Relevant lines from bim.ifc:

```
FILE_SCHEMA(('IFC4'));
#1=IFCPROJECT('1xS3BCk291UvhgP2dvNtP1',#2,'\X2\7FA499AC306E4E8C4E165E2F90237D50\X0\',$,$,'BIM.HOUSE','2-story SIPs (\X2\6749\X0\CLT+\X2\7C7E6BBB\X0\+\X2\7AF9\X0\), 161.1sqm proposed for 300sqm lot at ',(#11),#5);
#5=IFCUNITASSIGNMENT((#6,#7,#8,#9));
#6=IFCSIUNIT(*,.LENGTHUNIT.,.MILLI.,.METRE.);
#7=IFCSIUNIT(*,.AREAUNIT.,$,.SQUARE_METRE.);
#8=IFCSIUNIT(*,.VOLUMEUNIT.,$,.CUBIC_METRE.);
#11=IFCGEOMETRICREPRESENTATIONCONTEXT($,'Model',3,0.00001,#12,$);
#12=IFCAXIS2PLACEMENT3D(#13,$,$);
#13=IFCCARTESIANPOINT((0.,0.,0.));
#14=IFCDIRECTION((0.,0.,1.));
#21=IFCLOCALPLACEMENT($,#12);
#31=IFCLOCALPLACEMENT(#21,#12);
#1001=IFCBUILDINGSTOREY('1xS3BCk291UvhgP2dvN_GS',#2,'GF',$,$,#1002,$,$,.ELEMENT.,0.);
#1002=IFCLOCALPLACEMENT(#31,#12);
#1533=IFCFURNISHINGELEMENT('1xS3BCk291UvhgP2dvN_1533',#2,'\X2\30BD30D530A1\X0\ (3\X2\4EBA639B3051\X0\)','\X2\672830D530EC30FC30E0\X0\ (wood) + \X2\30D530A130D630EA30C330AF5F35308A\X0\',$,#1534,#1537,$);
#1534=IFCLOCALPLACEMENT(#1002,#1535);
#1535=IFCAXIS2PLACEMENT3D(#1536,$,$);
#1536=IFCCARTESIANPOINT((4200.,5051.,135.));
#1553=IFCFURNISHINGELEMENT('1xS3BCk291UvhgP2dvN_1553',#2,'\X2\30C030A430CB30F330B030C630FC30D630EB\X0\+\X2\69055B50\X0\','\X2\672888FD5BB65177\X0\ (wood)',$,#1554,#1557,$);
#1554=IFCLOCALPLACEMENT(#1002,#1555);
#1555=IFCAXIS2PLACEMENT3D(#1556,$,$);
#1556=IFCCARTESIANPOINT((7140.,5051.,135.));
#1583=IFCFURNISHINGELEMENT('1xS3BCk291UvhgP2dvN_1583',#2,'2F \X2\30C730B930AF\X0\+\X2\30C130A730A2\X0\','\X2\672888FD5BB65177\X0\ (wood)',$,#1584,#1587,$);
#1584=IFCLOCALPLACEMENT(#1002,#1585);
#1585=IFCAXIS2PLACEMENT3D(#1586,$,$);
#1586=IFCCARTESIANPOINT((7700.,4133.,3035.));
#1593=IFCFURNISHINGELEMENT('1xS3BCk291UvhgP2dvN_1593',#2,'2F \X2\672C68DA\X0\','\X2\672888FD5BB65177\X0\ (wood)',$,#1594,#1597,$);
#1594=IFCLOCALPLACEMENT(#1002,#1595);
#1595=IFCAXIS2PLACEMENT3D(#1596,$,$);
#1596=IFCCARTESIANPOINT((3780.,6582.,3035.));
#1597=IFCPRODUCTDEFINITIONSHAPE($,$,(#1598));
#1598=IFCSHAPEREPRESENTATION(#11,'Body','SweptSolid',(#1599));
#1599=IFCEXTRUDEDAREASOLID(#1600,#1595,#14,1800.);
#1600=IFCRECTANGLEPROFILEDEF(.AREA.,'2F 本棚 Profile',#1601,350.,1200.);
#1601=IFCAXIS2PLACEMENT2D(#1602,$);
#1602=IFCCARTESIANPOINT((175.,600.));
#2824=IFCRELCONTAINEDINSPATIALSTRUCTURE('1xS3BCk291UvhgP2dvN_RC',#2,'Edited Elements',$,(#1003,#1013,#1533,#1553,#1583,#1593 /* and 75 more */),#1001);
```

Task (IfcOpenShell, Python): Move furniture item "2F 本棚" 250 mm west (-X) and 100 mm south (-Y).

```python
import ifcopenshell
import ifcopenshell.api.geometry
import ifcopenshell.util.placement
import ifcopenshell.util.unit

model = ifcopenshell.open("bim.ifc")
unit_scale = ifcopenshell.util.unit.calculate_unit_scale(model)

item = model.by_guid("1xS3BCk291UvhgP2dvN_1593")
matrix = ifcopenshell.util.placement.get_local_placement(item.ObjectPlacement)
matrix[0, 3] -= 0.25 / unit_scale
matrix[1, 3] -= 0.1 / unit_scale
ifcopenshell.api.geometry.edit_object_placement(model, product=item, matrix=matrix, is_si=False)

print(ifcopenshell.util.placement.get_local_placement(item.ObjectPlacement).round(3) + 0.0)

model.write("bim_v2.ifc")
```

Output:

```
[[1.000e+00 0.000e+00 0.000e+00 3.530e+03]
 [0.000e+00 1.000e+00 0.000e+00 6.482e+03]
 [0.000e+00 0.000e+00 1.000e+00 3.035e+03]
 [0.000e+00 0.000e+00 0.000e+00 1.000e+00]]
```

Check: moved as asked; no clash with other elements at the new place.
